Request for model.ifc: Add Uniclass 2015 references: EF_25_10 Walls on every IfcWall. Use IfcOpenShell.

First a look at what the model holds.

```python
import ifcopenshell

model = ifcopenshell.open("model.ifc")
print(model.schema)
print("classifications:", [c.Name for c in model.by_type("IfcClassification")])
for ifc_class in ("IfcDoor", "IfcRoof", "IfcStair", "IfcWall", "IfcWindow"):
    print(ifc_class, len(model.by_type(ifc_class)))
```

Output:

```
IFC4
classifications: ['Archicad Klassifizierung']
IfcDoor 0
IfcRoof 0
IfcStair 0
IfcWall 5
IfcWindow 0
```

```python
import ifcopenshell
import ifcopenshell.api.classification

model = ifcopenshell.open("model.ifc")

system = ifcopenshell.api.classification.add_classification(model, classification="Uniclass 2015")

codes = {
    "IfcWall": ("EF_25_10", "Walls"),
}
for ifc_class, (code, name) in codes.items():
    products = model.by_type(ifc_class)
    ifcopenshell.api.classification.add_reference(
        model, products=products, classification=system, identification=code, name=name
    )
    print(code, len(products))

model.write("model_edited.ifc")
```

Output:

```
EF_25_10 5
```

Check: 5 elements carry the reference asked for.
